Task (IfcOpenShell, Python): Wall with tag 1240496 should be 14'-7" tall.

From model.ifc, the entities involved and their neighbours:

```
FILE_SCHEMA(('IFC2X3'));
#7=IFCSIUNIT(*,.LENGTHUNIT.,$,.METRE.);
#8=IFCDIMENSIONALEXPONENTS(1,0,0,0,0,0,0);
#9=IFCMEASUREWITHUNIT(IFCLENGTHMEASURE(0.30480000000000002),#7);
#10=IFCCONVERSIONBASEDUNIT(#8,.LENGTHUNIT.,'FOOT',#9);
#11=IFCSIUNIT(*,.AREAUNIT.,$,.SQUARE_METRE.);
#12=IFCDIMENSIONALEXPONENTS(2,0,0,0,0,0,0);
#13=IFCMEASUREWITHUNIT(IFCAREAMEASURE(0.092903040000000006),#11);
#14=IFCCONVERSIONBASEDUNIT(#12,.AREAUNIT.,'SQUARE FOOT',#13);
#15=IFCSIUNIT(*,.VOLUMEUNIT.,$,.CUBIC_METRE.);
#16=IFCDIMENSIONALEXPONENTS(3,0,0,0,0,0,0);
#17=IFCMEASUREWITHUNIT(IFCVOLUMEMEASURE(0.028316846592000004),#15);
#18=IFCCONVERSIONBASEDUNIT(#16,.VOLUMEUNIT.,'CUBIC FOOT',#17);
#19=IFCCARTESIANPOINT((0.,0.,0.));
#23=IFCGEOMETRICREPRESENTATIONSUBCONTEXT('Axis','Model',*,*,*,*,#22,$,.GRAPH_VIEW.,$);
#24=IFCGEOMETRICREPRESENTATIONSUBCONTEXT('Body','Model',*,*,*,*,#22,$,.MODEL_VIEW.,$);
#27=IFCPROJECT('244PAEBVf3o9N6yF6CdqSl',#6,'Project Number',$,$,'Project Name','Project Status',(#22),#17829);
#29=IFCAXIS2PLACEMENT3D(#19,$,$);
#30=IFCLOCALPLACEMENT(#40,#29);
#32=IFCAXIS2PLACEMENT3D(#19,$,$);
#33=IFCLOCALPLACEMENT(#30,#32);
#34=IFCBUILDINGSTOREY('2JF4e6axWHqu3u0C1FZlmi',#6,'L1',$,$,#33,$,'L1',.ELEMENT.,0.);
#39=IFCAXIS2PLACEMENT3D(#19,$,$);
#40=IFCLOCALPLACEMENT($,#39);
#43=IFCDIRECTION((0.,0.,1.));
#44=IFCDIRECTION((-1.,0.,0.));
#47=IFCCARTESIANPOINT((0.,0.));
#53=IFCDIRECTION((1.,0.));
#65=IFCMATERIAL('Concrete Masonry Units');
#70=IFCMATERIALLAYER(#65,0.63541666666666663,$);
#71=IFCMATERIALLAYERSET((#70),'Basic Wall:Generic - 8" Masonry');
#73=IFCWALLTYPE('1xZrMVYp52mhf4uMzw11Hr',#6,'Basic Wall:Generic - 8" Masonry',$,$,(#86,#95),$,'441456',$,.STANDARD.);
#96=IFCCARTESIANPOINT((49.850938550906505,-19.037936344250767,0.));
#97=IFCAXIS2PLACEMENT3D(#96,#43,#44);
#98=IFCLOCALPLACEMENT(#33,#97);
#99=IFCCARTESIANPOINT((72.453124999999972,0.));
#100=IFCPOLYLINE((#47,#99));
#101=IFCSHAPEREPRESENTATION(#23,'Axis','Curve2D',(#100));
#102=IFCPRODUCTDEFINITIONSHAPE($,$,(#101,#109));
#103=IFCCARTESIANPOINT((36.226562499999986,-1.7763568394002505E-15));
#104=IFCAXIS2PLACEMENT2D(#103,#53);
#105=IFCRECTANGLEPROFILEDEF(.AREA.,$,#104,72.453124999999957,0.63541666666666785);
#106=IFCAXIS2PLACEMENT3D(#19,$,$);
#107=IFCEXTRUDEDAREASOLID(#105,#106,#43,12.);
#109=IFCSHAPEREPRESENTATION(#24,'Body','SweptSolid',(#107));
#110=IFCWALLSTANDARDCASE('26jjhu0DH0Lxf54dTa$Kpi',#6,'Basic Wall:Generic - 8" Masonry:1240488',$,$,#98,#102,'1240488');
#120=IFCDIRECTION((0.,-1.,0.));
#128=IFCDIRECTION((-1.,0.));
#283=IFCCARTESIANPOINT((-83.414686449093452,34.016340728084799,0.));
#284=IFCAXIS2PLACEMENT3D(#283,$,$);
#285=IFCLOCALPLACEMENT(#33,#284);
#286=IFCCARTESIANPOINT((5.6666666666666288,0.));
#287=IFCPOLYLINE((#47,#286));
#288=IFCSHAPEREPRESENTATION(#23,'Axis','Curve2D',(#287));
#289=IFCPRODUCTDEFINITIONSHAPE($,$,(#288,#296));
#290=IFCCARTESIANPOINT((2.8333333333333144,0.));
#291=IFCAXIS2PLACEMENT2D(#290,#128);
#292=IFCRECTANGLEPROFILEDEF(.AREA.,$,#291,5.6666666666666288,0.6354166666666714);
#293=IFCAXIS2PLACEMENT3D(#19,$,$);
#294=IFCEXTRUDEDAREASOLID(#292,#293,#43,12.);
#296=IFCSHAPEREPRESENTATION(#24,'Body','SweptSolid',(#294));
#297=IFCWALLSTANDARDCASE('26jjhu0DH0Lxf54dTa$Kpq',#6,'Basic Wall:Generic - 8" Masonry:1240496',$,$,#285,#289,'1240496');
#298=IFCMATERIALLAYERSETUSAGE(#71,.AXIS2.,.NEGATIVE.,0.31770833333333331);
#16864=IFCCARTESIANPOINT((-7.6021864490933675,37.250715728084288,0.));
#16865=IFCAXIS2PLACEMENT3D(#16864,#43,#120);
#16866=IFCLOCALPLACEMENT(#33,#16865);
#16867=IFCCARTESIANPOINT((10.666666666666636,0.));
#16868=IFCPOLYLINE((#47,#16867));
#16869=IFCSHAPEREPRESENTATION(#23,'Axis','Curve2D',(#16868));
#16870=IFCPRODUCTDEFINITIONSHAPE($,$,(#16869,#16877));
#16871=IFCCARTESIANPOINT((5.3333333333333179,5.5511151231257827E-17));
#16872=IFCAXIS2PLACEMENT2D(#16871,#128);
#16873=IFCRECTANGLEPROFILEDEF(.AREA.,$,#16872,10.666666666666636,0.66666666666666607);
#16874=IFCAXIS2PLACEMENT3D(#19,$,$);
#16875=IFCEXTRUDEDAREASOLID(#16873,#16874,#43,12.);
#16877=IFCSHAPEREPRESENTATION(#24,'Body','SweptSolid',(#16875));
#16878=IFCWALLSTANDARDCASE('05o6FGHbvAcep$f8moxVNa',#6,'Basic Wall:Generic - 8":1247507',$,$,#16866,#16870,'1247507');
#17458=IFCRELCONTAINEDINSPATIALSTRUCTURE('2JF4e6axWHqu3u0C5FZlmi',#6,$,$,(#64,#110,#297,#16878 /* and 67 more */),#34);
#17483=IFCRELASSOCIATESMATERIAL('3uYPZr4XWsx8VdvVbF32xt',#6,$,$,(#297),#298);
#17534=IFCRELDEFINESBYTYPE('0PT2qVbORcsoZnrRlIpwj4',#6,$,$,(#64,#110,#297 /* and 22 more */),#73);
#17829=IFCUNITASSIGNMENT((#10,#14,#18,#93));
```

```python
import ifcopenshell
import ifcopenshell.geom
import ifcopenshell.util.representation
import ifcopenshell.util.shape
import ifcopenshell.util.unit

model = ifcopenshell.open("model.ifc")
unit_scale = ifcopenshell.util.unit.calculate_unit_scale(model)
settings = ifcopenshell.geom.settings()


def volume(element):
    """Net volume in cubic metres, openings subtracted."""
    shape = ifcopenshell.geom.create_shape(settings, element)
    return ifcopenshell.util.shape.get_volume(shape.geometry)


wall = model.by_id(297)
before = volume(wall)

body = ifcopenshell.util.representation.get_representation(wall, "Model", "Body")
solid = body.Items[0]
old_height = solid.Depth
solid.Depth = 175 * 0.0254 / unit_scale
after = volume(wall)

print(f"height {old_height:g} -> {solid.Depth:g}, volume {before:.3f} -> {after:.3f} m3")

model.write("model_rev.ifc")
```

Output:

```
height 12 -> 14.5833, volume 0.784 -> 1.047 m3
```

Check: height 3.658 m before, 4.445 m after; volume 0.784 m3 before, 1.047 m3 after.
